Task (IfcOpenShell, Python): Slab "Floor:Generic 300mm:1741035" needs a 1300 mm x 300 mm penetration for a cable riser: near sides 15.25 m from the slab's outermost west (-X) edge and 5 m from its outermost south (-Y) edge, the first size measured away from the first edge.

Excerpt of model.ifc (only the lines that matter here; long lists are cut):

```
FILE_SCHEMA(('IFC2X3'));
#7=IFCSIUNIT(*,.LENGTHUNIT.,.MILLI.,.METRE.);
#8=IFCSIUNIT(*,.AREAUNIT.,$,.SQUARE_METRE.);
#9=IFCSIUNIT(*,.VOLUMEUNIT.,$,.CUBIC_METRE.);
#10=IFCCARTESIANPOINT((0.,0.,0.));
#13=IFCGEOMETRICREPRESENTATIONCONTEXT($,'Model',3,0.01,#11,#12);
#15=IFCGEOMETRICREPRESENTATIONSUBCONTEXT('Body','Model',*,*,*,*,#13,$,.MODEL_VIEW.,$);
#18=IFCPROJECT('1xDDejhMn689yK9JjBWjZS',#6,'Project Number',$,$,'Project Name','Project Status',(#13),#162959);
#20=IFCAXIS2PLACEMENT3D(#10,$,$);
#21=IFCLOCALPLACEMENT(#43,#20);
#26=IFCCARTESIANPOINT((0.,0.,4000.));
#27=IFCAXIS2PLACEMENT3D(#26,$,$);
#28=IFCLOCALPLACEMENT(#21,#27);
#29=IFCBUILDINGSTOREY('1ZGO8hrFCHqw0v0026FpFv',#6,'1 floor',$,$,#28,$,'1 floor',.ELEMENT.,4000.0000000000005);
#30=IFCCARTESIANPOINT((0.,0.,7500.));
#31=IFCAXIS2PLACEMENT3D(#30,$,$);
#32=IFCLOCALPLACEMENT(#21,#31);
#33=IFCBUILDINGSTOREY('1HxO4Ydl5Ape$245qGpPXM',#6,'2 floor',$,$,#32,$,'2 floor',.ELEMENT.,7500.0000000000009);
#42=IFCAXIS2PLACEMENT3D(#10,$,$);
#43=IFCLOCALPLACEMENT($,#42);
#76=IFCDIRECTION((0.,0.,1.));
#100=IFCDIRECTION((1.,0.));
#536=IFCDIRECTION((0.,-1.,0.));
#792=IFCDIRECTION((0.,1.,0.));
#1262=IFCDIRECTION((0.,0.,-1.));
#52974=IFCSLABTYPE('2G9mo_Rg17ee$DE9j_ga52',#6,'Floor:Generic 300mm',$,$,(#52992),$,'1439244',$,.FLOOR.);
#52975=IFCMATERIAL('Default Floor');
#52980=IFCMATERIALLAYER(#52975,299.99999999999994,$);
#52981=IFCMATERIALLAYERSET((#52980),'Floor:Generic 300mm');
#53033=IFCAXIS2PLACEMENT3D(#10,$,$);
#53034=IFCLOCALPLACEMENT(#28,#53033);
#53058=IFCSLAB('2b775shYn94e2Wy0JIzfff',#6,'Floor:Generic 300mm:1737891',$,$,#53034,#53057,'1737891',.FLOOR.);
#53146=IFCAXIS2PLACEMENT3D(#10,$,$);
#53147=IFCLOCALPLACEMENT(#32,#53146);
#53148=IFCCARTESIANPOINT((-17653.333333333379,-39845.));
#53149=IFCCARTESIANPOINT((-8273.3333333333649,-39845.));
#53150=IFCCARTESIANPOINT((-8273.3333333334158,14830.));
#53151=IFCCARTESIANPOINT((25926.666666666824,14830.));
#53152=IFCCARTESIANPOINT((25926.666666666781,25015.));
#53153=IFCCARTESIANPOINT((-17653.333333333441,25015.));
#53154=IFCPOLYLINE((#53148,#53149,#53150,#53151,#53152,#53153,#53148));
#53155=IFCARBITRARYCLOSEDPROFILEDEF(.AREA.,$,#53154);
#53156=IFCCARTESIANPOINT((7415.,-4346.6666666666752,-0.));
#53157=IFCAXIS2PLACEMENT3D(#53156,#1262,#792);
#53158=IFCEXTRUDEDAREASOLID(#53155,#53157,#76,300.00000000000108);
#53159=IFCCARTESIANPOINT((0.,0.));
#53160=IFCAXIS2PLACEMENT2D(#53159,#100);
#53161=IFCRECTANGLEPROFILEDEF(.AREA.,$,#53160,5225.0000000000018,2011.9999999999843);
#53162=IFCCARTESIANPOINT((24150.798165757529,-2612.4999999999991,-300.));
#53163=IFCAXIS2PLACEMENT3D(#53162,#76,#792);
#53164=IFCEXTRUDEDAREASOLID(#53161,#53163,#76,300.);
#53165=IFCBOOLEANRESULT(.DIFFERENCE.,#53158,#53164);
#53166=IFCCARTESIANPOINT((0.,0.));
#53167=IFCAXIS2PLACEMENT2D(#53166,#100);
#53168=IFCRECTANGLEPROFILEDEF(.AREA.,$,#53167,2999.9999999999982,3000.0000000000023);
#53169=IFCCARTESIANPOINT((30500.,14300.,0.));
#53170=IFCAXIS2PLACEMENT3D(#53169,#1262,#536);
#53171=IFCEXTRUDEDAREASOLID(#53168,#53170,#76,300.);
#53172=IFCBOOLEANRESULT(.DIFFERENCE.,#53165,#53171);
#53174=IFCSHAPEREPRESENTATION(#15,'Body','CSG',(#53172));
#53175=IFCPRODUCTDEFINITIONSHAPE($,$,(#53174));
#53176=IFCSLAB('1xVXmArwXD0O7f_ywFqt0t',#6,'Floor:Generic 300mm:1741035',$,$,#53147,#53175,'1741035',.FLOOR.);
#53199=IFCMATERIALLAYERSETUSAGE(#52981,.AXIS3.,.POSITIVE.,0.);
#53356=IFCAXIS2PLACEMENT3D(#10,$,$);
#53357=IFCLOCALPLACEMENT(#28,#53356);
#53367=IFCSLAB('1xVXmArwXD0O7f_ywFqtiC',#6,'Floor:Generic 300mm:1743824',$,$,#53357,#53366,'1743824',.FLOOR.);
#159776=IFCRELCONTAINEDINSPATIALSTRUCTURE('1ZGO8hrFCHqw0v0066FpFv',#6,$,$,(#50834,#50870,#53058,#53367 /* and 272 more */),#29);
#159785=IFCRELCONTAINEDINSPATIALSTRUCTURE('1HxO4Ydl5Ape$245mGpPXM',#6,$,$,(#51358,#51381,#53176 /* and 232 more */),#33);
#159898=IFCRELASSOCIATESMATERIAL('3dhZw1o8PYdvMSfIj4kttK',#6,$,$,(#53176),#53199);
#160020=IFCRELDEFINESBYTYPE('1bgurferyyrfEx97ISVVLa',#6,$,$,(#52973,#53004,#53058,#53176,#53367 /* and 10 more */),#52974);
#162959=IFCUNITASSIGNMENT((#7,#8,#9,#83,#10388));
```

```python
import numpy as np
import ifcopenshell
import ifcopenshell.api.feature
import ifcopenshell.api.geometry
import ifcopenshell.api.root
import ifcopenshell.geom
import ifcopenshell.util.placement
import ifcopenshell.util.representation
import ifcopenshell.util.shape
import ifcopenshell.util.unit

model = ifcopenshell.open("model.ifc")
unit_scale = ifcopenshell.util.unit.calculate_unit_scale(model)
settings = ifcopenshell.geom.settings()


def volume(element):
    """Net volume in cubic metres, openings subtracted."""
    shape = ifcopenshell.geom.create_shape(settings, element)
    return ifcopenshell.util.shape.get_volume(shape.geometry)


slab = model.by_guid("1xVXmArwXD0O7f_ywFqt0t")
before = volume(slab)

# Extent in the slab's own axes, in metres. The edges named are its -X and -Y sides.
slab_shape = ifcopenshell.geom.create_shape(settings, slab)
vertices = ifcopenshell.util.shape.get_vertices(slab_shape.geometry)
x_min, y_min, bottom = vertices.min(axis=0)
top = vertices[:, 2].max()

opening = ifcopenshell.api.root.create_entity(model, ifc_class="IfcOpeningElement", name="Cable riser opening")
context = ifcopenshell.util.representation.get_context(model, "Model", "Body", "MODEL_VIEW")
width, depth = 1.3, 0.3
outline = [(0.0, 0.0), (width, 0.0), (width, depth), (0.0, depth), (0.0, 0.0)]
# Overshoot both faces by 50 mm so the cut is clean.
shape = ifcopenshell.api.geometry.add_slab_representation(
    model, context=context, depth=top - bottom + 0.1, polyline=outline
)
ifcopenshell.api.geometry.assign_representation(model, product=opening, representation=shape)

matrix = ifcopenshell.util.placement.get_local_placement(slab.ObjectPlacement)
matrix[:, 3] = matrix @ np.append(np.array([x_min + 15.25, y_min + 5, bottom - 0.05]) / unit_scale, 1.0)
ifcopenshell.api.geometry.edit_object_placement(model, product=opening, matrix=matrix, is_si=False)
ifcopenshell.api.feature.add_feature(model, feature=opening, element=slab)

after = volume(slab)

print(f"slab volume {before:.3f} -> {after:.3f} m3")

model.write("model_rev.ifc")
```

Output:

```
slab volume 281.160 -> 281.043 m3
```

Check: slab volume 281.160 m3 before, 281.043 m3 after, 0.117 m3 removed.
